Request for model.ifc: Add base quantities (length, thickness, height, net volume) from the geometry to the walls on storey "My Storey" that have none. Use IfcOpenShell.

First a look at what the model holds.

```python
import ifcopenshell
import ifcopenshell.util.element
import ifcopenshell.util.unit

model = ifcopenshell.open("model.ifc")
print(model.schema)
for unit_type in ("LENGTHUNIT", "AREAUNIT", "VOLUMEUNIT"):
    print(unit_type, ifcopenshell.util.unit.calculate_unit_scale(model, unit_type))
storey = next(s for s in model.by_type("IfcBuildingStorey") if s.Name == "My Storey")
walls = [e for e in ifcopenshell.util.element.get_decomposition(storey) if e.is_a("IfcWall")]
for e in sorted(walls, key=lambda e: e.id()):
    print(e.id(), e.is_a(), e.Name, list(ifcopenshell.util.element.get_psets(e, qtos_only=True)), sep=" | ")
```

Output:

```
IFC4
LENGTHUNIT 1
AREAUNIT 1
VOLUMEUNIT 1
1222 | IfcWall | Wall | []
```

```python
import ifcopenshell
import ifcopenshell.api.pset
import ifcopenshell.geom
import ifcopenshell.util.element
import ifcopenshell.util.shape
import ifcopenshell.util.unit

model = ifcopenshell.open("model.ifc")
unit_scale = ifcopenshell.util.unit.calculate_unit_scale(model)
volume_scale = ifcopenshell.util.unit.calculate_unit_scale(model, "VOLUMEUNIT")
settings = ifcopenshell.geom.settings()

storey = next(s for s in model.by_type("IfcBuildingStorey") if s.Name == "My Storey")
walls = [e for e in ifcopenshell.util.element.get_decomposition(storey) if e.is_a("IfcWall")]

for e in sorted(walls, key=lambda e: e.id()):
    if ifcopenshell.util.element.get_psets(e, qtos_only=True, should_inherit=False):
        continue
    # Geometry comes back in metres, in the element's own axes.
    shape = ifcopenshell.geom.create_shape(settings, e)
    values = {
        "Length": ifcopenshell.util.shape.get_x(shape.geometry) / unit_scale,
        "Width": ifcopenshell.util.shape.get_y(shape.geometry) / unit_scale,
        "Height": ifcopenshell.util.shape.get_z(shape.geometry) / unit_scale,
        "NetVolume": ifcopenshell.util.shape.get_volume(shape.geometry) / volume_scale,
    }
    qto = ifcopenshell.api.pset.add_qto(model, product=e, name="Qto_WallBaseQuantities")
    ifcopenshell.api.pset.edit_qto(model, qto=qto, properties=values)
    print(e.id(), {k: round(v, 3) for k, v in values.items()})

model.write("model_v2.ifc")
```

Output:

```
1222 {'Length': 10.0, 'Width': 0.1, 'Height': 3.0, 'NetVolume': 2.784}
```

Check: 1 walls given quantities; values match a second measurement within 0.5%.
